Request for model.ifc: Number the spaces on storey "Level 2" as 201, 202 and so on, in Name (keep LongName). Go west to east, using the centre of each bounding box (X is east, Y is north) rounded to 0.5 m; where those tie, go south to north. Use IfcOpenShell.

First a look at what the model holds.

```python
import ifcopenshell
import ifcopenshell.util.element
import ifcopenshell.util.placement

model = ifcopenshell.open("model.ifc")
print(model.schema)
storey = next(s for s in model.by_type("IfcBuildingStorey") if s.Name == "Level 2")
spaces = [e for e in ifcopenshell.util.element.get_decomposition(storey) if e.is_a("IfcSpace")]
for e in sorted(spaces, key=lambda e: e.id()):
    origin = ifcopenshell.util.placement.get_local_placement(e.ObjectPlacement)[:3, 3]
    print(e.id(), e.Name, e.LongName, origin.round(2) + 0.0, sep=" | ")
```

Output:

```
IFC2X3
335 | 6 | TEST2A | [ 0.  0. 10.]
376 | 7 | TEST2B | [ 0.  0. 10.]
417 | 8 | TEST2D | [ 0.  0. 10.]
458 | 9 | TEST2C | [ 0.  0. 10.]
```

```python
import ifcopenshell
import ifcopenshell.geom
import ifcopenshell.util.element
import ifcopenshell.util.shape

model = ifcopenshell.open("model.ifc")
settings = ifcopenshell.geom.settings()
settings.set("use-world-coords", True)


def centre(element):
    shape = ifcopenshell.geom.create_shape(settings, element)
    return ifcopenshell.util.shape.get_bbox_centroid(shape.geometry)


storey = next(s for s in model.by_type("IfcBuildingStorey") if s.Name == "Level 2")
spaces = [e for e in ifcopenshell.util.element.get_decomposition(storey) if e.is_a("IfcSpace")]

# Insertion points can sit at a corner or the storey origin, so sort by the geometry (in metres).
centres = {e: centre(e) for e in spaces}
spaces.sort(key=lambda e: (round(centres[e][0] / 0.5), centres[e][1]))

for i, e in enumerate(spaces, start=1):
    number = f"2{i:02d}"
    e.Name = number
    print(e.id(), number)

model.write("model_updated.ifc")
```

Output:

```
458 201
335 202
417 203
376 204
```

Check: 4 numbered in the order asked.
